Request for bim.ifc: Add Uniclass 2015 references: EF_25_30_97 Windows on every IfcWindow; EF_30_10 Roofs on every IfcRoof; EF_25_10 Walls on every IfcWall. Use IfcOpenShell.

First a look at what the model holds.

```python
import ifcopenshell

model = ifcopenshell.open("bim.ifc")
print(model.schema)
print("classifications:", [c.Name for c in model.by_type("IfcClassification")])
for ifc_class in ("IfcDoor", "IfcRoof", "IfcStair", "IfcWall", "IfcWindow"):
    print(ifc_class, len(model.by_type(ifc_class)))
```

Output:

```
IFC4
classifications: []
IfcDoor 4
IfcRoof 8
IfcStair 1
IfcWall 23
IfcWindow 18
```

```python
import ifcopenshell
import ifcopenshell.api.classification

model = ifcopenshell.open("bim.ifc")

system = ifcopenshell.api.classification.add_classification(model, classification="Uniclass 2015")

codes = {
    "IfcWindow": ("EF_25_30_97", "Windows"),
    "IfcRoof": ("EF_30_10", "Roofs"),
    "IfcWall": ("EF_25_10", "Walls"),
}
for ifc_class, (code, name) in codes.items():
    products = model.by_type(ifc_class)
    ifcopenshell.api.classification.add_reference(
        model, products=products, classification=system, identification=code, name=name
    )
    print(code, len(products))

model.write("bim_updated.ifc")
```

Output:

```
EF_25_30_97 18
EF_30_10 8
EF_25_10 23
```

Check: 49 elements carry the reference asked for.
